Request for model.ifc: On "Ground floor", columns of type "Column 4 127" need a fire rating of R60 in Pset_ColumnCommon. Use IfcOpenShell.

First a look at what the model holds.

```python
import ifcopenshell
import ifcopenshell.util.element

model = ifcopenshell.open("model.ifc")
print(model.schema)
storey = next(s for s in model.by_type("IfcBuildingStorey") if s.Name == "Ground floor")
columns = [e for e in ifcopenshell.util.element.get_decomposition(storey) if e.is_a("IfcColumn")]
seen = {}
for e in columns:
    element_type = ifcopenshell.util.element.get_type(e)
    key = (element_type.Name if element_type != e and element_type else None, ifcopenshell.util.element.get_pset(e, "Pset_ColumnCommon", "FireRating"))
    seen[key] = seen.get(key, 0) + 1
for (name, value), count in sorted(seen.items(), key=str):
    print(count, "x", name, "|", value)
```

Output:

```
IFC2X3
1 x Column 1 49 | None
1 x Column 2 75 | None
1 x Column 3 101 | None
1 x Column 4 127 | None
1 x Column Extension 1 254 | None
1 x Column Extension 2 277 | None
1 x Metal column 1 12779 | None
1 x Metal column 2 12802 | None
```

```python
import ifcopenshell
import ifcopenshell.api.pset
import ifcopenshell.util.element

model = ifcopenshell.open("model.ifc")

storey = next(s for s in model.by_type("IfcBuildingStorey") if s.Name == "Ground floor")
columns = [e for e in ifcopenshell.util.element.get_decomposition(storey) if e.is_a("IfcColumn")]

count = 0
for e in columns:
    element_type = ifcopenshell.util.element.get_type(e)
    if element_type in (None, e) or element_type.Name != "Column 4 127":
        continue
    # add_pset returns the element's existing set when there is one.
    pset = ifcopenshell.api.pset.add_pset(model, product=e, name="Pset_ColumnCommon")
    ifcopenshell.api.pset.edit_pset(model, pset=pset, properties={"FireRating": "R60"})
    count += 1

print(count, "columns updated")

model.write("model-out.ifc")
```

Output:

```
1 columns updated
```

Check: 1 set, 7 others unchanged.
